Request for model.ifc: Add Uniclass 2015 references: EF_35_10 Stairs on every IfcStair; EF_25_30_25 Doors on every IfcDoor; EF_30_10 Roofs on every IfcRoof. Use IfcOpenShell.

First a look at what the model holds.

```python
import ifcopenshell

model = ifcopenshell.open("model.ifc")
print(model.schema)
print("classifications:", [c.Name for c in model.by_type("IfcClassification")])
for ifc_class in ("IfcDoor", "IfcRoof", "IfcStair", "IfcWall", "IfcWindow"):
    print(ifc_class, len(model.by_type(ifc_class)))
```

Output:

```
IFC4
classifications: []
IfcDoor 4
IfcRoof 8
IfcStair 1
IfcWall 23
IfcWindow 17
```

```python
import ifcopenshell
import ifcopenshell.api.classification

model = ifcopenshell.open("model.ifc")

system = ifcopenshell.api.classification.add_classification(model, classification="Uniclass 2015")

codes = {
    "IfcStair": ("EF_35_10", "Stairs"),
    "IfcDoor": ("EF_25_30_25", "Doors"),
    "IfcRoof": ("EF_30_10", "Roofs"),
}
for ifc_class, (code, name) in codes.items():
    products = model.by_type(ifc_class)
    ifcopenshell.api.classification.add_reference(
        model, products=products, classification=system, identification=code, name=name
    )
    print(code, len(products))

model.write("model_rev.ifc")
```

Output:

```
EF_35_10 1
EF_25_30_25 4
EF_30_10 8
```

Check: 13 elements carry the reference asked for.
